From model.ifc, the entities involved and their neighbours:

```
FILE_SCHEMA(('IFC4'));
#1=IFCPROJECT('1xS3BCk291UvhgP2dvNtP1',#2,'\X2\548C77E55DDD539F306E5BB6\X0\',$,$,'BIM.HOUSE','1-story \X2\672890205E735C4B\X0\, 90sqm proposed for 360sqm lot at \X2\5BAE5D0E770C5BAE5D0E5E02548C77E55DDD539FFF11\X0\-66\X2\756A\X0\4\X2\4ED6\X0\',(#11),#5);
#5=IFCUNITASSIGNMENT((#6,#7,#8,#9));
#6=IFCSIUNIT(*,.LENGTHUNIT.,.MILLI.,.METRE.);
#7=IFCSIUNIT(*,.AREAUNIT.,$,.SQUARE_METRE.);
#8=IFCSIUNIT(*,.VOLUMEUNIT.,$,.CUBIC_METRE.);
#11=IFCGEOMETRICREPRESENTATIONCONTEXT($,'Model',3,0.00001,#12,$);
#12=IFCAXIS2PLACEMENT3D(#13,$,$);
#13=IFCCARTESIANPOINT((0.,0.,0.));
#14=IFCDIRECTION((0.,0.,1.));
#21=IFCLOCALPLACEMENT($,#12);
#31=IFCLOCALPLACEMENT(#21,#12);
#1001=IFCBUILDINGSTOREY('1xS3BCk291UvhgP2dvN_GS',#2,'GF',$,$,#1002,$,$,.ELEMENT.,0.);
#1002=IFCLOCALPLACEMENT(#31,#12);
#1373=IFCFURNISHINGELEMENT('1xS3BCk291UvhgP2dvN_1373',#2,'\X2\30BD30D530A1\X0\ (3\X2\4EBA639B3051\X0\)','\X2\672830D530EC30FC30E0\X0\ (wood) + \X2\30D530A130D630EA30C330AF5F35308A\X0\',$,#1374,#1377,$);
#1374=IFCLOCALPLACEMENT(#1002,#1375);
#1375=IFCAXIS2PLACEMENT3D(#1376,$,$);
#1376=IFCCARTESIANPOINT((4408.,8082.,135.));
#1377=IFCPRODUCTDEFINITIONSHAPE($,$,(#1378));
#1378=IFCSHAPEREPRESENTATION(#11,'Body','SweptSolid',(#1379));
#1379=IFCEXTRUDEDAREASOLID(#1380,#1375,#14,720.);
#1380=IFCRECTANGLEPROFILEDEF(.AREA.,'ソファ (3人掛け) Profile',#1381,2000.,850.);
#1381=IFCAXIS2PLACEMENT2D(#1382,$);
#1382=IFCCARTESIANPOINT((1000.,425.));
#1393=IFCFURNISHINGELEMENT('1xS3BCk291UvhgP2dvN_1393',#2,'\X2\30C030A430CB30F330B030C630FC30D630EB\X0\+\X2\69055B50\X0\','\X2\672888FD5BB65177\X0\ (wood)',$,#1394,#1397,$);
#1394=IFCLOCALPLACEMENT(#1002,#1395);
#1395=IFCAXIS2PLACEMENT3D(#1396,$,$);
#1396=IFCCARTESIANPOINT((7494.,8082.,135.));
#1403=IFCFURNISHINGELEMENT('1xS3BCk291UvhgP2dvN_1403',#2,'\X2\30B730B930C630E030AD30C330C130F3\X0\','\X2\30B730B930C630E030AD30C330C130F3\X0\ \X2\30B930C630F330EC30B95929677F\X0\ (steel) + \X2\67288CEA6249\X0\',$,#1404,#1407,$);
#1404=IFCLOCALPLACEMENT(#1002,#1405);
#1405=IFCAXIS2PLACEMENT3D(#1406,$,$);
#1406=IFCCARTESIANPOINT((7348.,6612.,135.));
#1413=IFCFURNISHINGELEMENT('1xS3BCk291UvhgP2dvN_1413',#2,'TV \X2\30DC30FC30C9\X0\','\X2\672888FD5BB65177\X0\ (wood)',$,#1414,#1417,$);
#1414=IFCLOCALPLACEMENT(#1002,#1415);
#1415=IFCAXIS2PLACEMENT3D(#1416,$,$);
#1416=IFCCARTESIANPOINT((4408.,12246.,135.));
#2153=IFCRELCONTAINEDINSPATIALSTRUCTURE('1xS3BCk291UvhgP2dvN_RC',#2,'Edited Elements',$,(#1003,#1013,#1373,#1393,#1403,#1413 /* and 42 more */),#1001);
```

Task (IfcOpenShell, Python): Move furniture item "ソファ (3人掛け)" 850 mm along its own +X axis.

```python
import ifcopenshell
import ifcopenshell.api.geometry
import ifcopenshell.util.placement
import ifcopenshell.util.unit

model = ifcopenshell.open("model.ifc")
unit_scale = ifcopenshell.util.unit.calculate_unit_scale(model)

item = model.by_guid("1xS3BCk291UvhgP2dvN_1373")
matrix = ifcopenshell.util.placement.get_local_placement(item.ObjectPlacement)
matrix[:3, 3] += matrix[:3, 0] * 0.85 / unit_scale
ifcopenshell.api.geometry.edit_object_placement(model, product=item, matrix=matrix, is_si=False)

print(ifcopenshell.util.placement.get_local_placement(item.ObjectPlacement).round(3) + 0.0)

model.write("model_v2.ifc")
```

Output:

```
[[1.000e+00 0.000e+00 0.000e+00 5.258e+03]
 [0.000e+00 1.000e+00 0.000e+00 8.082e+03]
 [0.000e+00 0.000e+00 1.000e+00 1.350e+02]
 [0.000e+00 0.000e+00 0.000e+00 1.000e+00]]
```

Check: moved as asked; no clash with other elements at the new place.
